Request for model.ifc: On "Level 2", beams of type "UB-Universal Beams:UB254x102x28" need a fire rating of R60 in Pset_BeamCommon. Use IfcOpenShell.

First a look at what the model holds.

```python
import ifcopenshell
import ifcopenshell.util.element

model = ifcopenshell.open("model.ifc")
print(model.schema)
storey = next(s for s in model.by_type("IfcBuildingStorey") if s.Name == "Level 2")
beams = [e for e in ifcopenshell.util.element.get_decomposition(storey) if e.is_a("IfcBeam")]
seen = {}
for e in beams:
    element_type = ifcopenshell.util.element.get_type(e)
    key = (element_type.Name if element_type != e and element_type else None, ifcopenshell.util.element.get_pset(e, "Pset_BeamCommon", "FireRating"))
    seen[key] = seen.get(key, 0) + 1
for (name, value), count in sorted(seen.items(), key=str):
    print(count, "x", name, "|", value)
```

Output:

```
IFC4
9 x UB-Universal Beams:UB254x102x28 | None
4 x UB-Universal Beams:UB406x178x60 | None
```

```python
import ifcopenshell
import ifcopenshell.api.pset
import ifcopenshell.util.element

model = ifcopenshell.open("model.ifc")

storey = next(s for s in model.by_type("IfcBuildingStorey") if s.Name == "Level 2")
beams = [e for e in ifcopenshell.util.element.get_decomposition(storey) if e.is_a("IfcBeam")]

count = 0
for e in beams:
    element_type = ifcopenshell.util.element.get_type(e)
    if element_type in (None, e) or element_type.Name != "UB-Universal Beams:UB254x102x28":
        continue
    # add_pset returns the element's existing set when there is one.
    pset = ifcopenshell.api.pset.add_pset(model, product=e, name="Pset_BeamCommon")
    ifcopenshell.api.pset.edit_pset(model, pset=pset, properties={"FireRating": "R60"})
    count += 1

print(count, "beams updated")

model.write("model-out.ifc")
```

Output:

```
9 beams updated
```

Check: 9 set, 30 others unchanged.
